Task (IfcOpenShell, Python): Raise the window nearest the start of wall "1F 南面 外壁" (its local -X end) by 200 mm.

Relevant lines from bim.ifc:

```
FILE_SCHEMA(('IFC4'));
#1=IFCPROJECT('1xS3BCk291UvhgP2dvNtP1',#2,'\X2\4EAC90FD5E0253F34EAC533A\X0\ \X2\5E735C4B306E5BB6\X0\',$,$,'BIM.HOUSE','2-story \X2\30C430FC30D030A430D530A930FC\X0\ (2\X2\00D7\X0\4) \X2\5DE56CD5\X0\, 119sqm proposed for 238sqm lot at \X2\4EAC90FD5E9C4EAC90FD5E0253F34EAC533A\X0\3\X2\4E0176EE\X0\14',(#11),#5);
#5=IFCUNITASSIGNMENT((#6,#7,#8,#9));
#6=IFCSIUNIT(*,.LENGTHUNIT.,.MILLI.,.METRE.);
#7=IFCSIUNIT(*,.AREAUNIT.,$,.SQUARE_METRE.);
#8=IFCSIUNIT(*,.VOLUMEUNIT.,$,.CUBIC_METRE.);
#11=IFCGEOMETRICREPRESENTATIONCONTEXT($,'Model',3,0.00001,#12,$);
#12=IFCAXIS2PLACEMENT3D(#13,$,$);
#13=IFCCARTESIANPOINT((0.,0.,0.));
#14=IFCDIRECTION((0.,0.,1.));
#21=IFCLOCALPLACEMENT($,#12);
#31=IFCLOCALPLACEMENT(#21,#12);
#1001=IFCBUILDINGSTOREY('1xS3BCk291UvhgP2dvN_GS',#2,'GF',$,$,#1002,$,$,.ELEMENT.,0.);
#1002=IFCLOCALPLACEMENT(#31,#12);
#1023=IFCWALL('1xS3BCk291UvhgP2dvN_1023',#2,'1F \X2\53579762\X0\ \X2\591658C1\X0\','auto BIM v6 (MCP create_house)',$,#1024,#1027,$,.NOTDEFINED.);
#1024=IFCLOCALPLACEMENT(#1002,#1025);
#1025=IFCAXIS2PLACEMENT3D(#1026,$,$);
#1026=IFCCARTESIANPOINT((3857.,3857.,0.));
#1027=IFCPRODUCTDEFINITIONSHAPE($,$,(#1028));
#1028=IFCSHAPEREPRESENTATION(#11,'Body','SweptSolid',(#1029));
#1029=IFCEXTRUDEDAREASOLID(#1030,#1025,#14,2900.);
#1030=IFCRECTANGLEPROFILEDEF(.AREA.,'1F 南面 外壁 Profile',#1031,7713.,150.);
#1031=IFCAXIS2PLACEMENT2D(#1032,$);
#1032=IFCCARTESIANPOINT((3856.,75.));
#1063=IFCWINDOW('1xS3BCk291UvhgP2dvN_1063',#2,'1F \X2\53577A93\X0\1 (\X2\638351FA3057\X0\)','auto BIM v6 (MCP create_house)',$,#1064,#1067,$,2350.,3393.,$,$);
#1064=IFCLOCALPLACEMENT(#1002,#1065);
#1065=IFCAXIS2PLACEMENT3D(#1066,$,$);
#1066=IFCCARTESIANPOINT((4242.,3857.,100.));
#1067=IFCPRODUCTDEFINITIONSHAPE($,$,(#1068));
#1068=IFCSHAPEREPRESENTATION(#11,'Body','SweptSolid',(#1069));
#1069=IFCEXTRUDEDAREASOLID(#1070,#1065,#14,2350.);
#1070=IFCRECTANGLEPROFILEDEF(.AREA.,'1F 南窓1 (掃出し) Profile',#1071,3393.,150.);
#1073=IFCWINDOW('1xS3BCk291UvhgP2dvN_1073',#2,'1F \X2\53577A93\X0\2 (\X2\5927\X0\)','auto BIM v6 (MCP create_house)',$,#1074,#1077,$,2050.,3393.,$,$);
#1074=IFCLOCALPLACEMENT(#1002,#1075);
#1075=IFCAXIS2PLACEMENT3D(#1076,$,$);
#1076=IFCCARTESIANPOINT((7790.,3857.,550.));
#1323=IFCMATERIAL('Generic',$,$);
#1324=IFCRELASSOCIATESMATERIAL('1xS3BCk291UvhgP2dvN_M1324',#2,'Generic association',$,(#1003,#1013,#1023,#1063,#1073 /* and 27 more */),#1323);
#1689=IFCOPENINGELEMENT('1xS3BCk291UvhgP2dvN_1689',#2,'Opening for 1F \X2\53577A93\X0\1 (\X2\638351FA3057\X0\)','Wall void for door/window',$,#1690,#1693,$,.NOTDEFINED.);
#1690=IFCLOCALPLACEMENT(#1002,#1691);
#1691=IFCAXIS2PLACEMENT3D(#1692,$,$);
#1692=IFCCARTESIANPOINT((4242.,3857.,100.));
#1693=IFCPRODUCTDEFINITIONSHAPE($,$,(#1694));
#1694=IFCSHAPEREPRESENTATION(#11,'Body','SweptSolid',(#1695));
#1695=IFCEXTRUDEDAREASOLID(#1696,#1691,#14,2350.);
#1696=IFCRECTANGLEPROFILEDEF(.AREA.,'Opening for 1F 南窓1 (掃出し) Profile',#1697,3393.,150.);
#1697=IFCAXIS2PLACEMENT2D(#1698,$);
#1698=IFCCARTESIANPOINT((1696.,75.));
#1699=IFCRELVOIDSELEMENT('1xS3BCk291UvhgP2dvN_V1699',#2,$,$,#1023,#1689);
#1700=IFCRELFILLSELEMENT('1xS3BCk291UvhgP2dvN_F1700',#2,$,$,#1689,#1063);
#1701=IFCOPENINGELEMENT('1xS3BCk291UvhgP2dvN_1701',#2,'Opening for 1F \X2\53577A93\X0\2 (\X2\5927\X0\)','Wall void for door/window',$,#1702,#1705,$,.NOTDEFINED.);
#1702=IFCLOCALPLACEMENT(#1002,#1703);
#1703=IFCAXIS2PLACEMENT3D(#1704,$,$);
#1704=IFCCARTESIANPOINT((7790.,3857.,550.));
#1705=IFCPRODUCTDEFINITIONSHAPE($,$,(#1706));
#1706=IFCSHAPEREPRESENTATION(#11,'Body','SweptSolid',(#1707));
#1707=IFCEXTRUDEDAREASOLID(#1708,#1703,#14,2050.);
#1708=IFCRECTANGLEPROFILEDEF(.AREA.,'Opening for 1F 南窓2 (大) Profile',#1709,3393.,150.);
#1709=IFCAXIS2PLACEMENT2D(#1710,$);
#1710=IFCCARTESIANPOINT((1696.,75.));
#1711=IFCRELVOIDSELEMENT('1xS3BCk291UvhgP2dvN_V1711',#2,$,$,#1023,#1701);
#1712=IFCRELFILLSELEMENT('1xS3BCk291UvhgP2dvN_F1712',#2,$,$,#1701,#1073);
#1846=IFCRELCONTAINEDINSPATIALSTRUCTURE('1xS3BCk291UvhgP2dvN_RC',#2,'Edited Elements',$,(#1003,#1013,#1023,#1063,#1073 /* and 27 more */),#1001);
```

```python
import numpy as np
import ifcopenshell
import ifcopenshell.api.geometry
import ifcopenshell.util.placement
import ifcopenshell.util.unit

model = ifcopenshell.open("bim.ifc")
unit_scale = ifcopenshell.util.unit.calculate_unit_scale(model)

window = model.by_guid("1xS3BCk291UvhgP2dvN_1063")
opening = window.FillsVoids[0].RelatingOpeningElement
dz = 0.2 / unit_scale

shift = np.array([0.0, 0.0, dz])
# The window is not placed relative to its opening, so move both.
for product in (opening, window):
    matrix = ifcopenshell.util.placement.get_local_placement(product.ObjectPlacement)
    matrix[:3, 3] += shift
    ifcopenshell.api.geometry.edit_object_placement(model, product=product, matrix=matrix, is_si=False)

print(f"moved by {dz * unit_scale:+.3f} m")

model.write("bim_edited.ifc")
```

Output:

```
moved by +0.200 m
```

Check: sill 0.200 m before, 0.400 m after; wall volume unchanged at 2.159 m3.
